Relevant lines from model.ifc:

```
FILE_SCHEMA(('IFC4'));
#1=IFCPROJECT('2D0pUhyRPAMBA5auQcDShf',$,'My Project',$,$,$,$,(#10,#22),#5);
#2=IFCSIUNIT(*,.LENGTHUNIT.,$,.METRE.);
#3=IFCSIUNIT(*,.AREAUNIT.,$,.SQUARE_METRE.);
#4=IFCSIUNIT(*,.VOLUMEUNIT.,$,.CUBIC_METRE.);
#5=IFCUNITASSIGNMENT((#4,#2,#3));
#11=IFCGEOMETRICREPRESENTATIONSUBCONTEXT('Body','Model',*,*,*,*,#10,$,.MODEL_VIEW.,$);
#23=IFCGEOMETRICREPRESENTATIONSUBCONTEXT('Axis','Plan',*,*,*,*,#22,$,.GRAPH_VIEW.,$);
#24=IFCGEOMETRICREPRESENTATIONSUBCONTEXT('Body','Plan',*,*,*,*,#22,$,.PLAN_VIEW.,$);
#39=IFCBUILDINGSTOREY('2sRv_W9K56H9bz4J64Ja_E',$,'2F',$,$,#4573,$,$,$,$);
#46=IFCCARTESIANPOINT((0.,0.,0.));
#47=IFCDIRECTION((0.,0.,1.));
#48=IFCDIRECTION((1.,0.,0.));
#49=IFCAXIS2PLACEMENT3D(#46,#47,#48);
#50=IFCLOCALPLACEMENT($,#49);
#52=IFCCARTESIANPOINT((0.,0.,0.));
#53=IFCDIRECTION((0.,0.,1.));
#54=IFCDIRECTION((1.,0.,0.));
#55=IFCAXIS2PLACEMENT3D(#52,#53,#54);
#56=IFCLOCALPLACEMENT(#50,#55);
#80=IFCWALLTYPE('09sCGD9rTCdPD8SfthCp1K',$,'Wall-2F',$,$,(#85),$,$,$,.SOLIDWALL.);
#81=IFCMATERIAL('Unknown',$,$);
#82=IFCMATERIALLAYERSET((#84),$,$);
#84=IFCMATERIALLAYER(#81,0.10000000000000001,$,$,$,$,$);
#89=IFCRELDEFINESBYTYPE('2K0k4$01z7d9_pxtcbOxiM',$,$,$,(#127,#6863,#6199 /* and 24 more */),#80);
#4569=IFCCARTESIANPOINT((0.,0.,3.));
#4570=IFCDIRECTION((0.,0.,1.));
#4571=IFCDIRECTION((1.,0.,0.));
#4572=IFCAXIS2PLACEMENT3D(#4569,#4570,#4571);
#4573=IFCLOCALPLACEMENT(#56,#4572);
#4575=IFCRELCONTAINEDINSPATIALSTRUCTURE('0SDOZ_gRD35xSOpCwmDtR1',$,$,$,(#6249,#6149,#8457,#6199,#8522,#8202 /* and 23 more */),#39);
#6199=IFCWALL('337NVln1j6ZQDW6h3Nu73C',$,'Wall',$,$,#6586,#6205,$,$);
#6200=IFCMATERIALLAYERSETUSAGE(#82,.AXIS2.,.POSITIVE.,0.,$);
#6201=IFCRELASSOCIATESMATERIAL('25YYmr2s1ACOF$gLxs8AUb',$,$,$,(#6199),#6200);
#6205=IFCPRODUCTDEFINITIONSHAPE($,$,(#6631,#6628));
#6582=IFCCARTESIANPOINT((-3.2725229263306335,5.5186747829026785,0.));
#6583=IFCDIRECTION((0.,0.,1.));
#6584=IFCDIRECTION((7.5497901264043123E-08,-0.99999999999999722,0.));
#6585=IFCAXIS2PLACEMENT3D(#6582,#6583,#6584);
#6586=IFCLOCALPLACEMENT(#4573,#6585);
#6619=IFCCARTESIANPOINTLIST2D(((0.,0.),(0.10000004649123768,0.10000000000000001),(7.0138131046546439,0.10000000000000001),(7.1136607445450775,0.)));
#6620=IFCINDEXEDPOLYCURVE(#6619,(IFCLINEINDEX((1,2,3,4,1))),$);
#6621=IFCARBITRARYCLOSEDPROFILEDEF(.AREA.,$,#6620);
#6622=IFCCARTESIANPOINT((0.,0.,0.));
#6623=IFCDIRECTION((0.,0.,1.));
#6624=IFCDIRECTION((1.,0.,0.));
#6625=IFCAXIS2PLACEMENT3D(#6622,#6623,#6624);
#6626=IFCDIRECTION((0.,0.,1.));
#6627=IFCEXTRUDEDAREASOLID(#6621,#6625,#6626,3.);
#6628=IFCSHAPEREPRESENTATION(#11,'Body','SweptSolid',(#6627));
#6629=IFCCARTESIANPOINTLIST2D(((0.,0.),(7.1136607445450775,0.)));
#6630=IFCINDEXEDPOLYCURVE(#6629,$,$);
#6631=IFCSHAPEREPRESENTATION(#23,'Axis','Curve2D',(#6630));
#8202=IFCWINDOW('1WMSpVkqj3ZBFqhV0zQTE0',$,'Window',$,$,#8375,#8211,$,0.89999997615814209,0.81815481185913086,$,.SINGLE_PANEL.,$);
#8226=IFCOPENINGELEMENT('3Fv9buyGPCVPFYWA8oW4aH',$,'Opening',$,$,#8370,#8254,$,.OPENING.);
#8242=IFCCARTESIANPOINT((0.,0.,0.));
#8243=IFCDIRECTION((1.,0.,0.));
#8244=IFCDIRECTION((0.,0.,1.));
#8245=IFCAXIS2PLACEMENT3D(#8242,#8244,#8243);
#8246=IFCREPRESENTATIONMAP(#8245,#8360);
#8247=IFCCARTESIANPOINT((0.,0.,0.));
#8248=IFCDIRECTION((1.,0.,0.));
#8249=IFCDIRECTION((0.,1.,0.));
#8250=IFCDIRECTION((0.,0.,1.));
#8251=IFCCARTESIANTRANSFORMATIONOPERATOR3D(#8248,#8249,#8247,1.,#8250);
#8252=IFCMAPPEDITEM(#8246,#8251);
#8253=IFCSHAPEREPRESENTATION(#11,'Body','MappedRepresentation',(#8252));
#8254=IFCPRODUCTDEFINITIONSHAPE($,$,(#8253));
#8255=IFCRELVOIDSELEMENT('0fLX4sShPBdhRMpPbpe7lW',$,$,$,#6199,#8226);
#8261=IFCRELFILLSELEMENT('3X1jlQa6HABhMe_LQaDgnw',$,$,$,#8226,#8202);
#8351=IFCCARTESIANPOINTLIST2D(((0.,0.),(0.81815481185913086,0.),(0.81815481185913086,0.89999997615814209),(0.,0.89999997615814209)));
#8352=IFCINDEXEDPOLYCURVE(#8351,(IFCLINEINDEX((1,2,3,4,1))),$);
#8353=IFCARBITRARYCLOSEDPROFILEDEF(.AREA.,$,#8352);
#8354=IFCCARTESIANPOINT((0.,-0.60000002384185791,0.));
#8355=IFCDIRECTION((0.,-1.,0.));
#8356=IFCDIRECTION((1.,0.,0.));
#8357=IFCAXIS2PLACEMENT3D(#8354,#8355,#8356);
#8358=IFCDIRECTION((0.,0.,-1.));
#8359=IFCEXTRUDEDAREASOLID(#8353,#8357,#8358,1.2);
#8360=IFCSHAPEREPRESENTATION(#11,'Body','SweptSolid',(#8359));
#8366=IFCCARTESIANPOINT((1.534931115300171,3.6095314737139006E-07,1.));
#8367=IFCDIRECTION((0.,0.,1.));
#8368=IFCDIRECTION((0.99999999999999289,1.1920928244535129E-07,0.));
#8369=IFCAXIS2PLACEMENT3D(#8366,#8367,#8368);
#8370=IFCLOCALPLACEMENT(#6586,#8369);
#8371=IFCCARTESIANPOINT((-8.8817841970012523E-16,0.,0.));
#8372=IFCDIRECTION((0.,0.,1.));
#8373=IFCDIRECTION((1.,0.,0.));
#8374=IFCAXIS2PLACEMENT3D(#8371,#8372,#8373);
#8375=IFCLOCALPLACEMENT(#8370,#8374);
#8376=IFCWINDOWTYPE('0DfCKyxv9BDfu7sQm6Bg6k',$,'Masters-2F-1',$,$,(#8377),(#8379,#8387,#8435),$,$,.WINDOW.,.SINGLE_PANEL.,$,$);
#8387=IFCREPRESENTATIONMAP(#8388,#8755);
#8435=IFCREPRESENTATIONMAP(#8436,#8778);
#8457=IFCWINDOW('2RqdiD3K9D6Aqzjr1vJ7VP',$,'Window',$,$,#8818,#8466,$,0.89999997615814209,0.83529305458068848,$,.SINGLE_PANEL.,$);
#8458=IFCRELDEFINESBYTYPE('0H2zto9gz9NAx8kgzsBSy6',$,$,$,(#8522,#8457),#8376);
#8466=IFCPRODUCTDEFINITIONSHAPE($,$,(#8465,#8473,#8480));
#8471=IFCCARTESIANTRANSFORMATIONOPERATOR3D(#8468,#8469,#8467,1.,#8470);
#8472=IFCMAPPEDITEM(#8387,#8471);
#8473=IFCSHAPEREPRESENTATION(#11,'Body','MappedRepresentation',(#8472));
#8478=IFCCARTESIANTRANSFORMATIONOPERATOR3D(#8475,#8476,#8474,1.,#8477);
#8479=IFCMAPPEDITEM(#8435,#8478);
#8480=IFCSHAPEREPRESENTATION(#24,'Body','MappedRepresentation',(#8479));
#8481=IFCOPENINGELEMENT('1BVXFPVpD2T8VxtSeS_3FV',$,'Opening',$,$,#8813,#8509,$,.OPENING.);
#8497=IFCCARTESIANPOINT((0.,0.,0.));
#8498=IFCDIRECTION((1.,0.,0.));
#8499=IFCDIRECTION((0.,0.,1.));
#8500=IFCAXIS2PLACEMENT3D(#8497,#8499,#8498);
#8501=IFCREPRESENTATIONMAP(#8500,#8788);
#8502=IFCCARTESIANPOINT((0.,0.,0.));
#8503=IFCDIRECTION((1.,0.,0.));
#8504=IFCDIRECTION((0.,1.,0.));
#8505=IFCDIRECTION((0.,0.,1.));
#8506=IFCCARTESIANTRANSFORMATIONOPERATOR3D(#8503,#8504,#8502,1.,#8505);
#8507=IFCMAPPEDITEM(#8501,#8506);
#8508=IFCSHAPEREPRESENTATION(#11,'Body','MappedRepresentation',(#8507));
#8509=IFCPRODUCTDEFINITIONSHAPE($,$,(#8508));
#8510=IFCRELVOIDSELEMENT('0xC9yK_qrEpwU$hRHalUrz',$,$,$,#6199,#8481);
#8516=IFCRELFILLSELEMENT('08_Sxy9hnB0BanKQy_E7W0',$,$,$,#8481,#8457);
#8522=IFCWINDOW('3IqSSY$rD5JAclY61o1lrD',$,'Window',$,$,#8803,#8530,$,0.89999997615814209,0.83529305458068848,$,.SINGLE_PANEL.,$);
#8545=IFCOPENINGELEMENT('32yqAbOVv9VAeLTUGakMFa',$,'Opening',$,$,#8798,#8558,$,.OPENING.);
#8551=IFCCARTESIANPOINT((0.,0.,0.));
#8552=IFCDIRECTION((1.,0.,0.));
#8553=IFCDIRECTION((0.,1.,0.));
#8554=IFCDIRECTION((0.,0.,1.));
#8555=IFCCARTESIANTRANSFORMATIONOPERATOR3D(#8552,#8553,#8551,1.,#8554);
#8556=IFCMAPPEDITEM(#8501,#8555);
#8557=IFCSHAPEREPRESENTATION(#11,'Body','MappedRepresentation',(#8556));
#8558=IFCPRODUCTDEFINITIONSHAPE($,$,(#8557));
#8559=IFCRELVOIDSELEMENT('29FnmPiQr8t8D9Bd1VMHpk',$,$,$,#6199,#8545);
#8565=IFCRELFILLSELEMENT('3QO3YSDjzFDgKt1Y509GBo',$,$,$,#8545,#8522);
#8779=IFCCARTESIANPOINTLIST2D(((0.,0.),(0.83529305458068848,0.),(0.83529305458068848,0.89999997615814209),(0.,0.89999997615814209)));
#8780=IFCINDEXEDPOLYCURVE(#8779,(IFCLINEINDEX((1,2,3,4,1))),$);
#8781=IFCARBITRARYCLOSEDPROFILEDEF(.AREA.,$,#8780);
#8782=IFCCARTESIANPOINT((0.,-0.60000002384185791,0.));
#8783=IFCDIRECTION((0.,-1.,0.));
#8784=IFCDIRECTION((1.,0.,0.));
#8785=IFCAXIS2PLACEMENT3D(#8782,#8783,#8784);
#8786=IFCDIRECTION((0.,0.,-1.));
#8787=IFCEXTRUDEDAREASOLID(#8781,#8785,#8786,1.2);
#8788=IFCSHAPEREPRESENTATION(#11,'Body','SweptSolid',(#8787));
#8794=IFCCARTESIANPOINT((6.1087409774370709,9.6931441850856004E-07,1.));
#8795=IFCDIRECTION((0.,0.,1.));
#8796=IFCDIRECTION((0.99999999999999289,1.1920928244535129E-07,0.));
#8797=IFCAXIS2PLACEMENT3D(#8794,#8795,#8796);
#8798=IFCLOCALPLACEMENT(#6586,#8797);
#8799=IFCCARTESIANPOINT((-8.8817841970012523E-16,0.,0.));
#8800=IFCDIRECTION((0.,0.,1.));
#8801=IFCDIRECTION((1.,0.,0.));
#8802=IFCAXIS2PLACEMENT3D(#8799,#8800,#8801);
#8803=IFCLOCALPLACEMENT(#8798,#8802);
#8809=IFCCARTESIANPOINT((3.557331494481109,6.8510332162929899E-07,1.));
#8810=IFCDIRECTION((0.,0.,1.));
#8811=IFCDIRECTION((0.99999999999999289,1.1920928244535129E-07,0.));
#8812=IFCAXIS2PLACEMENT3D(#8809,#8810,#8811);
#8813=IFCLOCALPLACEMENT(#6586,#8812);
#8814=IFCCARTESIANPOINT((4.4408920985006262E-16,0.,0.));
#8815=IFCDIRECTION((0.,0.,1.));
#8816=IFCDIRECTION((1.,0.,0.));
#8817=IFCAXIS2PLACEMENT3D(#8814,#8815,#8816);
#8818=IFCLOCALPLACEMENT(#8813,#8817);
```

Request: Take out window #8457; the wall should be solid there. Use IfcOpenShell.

```python
import ifcopenshell
import ifcopenshell.api.feature
import ifcopenshell.api.root
import ifcopenshell.geom
import ifcopenshell.util.shape

model = ifcopenshell.open("model.ifc")
settings = ifcopenshell.geom.settings()


def volume(element):
    """Net volume in cubic metres, openings subtracted."""
    shape = ifcopenshell.geom.create_shape(settings, element)
    return ifcopenshell.util.shape.get_volume(shape.geometry)


window = model.by_id(8457)
opening = window.FillsVoids[0].RelatingOpeningElement
wall = opening.VoidsElements[0].RelatingBuildingElement
before = volume(wall)

ifcopenshell.api.root.remove_product(model, product=window)
ifcopenshell.api.feature.remove_feature(model, feature=opening)

after = volume(wall)

print(f"wall volume {before:.3f} -> {after:.3f} m3")

model.write("model_v2.ifc")
```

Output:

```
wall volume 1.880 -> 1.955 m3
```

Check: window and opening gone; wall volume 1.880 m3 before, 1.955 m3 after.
